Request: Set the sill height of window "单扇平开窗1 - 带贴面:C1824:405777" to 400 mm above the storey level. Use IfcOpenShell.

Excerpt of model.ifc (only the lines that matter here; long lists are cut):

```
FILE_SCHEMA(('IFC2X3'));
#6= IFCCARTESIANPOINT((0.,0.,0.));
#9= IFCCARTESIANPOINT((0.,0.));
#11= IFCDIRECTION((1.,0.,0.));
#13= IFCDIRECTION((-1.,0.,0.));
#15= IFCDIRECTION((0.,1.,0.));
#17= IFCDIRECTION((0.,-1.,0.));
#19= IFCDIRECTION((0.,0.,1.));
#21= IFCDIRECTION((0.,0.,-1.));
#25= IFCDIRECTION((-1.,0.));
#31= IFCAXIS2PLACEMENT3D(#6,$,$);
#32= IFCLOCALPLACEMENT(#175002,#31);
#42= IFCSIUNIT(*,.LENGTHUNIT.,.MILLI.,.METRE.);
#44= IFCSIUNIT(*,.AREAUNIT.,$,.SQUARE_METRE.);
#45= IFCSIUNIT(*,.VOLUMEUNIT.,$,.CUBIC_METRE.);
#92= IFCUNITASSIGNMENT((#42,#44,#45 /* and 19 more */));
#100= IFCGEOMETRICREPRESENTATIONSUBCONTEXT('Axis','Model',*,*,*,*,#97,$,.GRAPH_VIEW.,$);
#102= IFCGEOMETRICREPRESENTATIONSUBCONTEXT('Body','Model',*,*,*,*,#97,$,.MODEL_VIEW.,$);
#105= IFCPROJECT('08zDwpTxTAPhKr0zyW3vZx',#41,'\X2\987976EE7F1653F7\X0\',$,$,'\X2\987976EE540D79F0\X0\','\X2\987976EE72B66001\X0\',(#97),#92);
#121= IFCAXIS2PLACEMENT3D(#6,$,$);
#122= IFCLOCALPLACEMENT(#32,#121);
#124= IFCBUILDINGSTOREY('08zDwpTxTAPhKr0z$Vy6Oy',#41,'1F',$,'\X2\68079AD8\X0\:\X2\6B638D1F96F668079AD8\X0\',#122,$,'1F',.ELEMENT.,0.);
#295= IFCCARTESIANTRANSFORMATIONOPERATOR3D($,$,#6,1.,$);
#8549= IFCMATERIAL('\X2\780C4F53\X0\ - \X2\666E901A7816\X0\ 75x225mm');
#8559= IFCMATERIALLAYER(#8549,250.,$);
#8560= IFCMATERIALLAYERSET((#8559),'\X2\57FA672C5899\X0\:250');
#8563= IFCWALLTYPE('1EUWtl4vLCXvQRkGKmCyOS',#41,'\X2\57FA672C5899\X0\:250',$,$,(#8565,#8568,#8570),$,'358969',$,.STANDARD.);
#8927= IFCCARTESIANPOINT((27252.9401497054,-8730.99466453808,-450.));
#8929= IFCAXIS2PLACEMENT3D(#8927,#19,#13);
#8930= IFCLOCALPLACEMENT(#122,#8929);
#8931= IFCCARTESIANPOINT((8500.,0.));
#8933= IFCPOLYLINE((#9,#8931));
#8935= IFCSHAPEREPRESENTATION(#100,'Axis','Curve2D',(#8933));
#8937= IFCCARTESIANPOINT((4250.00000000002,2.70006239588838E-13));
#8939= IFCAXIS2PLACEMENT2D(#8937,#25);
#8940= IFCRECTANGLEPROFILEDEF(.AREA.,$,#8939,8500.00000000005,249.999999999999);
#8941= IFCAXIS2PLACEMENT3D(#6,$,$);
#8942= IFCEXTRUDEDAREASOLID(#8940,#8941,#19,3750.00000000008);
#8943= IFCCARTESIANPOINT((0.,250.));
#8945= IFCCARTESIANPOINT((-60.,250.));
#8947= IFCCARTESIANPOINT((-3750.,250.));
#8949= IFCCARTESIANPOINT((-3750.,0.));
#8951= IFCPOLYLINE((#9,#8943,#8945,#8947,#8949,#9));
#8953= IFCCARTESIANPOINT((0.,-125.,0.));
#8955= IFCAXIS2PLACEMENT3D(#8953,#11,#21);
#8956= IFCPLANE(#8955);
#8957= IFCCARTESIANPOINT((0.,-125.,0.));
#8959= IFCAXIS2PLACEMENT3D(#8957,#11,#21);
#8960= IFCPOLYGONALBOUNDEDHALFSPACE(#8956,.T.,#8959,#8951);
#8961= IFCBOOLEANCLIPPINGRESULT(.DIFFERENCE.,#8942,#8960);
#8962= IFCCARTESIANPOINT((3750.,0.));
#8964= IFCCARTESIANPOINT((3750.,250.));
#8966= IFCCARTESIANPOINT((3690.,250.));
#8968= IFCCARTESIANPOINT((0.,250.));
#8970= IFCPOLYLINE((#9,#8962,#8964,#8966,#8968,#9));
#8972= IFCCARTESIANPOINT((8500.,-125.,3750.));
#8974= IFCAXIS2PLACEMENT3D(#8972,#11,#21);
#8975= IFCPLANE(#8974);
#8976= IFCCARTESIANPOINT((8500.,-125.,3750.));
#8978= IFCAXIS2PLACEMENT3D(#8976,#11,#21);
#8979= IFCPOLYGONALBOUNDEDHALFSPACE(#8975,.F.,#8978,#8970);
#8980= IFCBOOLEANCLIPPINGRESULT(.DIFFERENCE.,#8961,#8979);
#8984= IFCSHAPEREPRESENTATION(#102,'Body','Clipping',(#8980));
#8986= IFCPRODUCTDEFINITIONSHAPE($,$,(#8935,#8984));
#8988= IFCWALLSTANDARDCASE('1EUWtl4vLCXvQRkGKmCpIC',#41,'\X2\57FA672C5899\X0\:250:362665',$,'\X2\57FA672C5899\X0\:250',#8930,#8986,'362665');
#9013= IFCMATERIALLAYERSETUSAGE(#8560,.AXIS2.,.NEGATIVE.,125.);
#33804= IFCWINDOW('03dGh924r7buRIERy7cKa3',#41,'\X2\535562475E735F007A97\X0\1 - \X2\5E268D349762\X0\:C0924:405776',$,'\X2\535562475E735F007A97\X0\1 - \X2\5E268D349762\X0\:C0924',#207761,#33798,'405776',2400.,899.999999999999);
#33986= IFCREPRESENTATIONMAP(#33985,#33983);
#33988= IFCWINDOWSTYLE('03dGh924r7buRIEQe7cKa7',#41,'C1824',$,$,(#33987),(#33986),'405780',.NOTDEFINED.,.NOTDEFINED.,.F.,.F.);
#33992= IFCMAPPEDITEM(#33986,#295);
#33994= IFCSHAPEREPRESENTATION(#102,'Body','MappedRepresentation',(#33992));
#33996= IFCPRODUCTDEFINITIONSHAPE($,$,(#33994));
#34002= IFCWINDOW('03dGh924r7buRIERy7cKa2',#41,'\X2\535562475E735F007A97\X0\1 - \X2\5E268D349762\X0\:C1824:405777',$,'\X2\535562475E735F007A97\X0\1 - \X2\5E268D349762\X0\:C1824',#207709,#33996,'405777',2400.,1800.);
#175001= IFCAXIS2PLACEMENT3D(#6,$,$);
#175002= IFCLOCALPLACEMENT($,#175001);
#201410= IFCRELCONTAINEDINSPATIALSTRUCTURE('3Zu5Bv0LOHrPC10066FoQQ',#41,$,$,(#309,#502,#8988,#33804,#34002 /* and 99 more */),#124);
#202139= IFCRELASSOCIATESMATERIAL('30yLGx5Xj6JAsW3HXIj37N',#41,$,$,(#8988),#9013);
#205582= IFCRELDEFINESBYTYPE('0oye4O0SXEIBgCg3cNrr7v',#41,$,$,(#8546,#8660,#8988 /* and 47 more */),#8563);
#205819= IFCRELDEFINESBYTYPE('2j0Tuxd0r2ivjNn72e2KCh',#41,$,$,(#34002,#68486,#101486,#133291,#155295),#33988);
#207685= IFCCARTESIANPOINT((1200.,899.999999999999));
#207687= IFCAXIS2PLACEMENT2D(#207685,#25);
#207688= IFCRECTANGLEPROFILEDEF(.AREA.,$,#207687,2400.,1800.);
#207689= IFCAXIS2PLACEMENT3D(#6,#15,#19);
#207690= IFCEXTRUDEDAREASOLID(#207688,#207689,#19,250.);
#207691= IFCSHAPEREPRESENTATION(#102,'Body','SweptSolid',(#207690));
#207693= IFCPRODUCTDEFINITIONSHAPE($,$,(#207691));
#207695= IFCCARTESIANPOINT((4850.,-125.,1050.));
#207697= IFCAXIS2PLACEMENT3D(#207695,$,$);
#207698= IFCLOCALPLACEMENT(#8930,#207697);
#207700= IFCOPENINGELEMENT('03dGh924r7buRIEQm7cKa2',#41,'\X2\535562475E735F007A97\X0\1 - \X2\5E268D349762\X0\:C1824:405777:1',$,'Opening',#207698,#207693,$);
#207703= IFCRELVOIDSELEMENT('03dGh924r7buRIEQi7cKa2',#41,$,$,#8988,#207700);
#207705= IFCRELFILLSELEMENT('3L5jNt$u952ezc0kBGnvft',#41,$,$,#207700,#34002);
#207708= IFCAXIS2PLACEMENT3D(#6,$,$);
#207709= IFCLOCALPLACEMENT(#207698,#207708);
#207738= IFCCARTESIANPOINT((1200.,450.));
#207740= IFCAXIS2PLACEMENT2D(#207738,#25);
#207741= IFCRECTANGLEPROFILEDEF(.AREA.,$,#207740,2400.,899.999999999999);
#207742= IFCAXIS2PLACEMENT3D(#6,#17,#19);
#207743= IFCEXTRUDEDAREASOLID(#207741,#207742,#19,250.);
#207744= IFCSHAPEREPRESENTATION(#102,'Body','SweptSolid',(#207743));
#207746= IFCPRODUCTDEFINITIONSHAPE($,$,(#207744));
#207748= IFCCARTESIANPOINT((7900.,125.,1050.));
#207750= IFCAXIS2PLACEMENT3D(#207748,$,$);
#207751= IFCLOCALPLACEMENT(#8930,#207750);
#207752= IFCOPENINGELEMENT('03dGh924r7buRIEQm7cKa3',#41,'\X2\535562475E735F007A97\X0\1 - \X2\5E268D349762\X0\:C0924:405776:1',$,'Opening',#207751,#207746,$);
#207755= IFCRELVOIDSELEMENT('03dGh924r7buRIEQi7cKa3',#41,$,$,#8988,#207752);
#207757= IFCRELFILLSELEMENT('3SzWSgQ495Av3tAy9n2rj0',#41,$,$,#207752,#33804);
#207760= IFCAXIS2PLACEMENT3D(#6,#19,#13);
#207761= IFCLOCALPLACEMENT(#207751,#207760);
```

```python
import numpy as np
import ifcopenshell
import ifcopenshell.api.geometry
import ifcopenshell.geom
import ifcopenshell.util.element
import ifcopenshell.util.placement
import ifcopenshell.util.shape
import ifcopenshell.util.unit

model = ifcopenshell.open("model.ifc")
unit_scale = ifcopenshell.util.unit.calculate_unit_scale(model)

window = model.by_id(34002)
opening = window.FillsVoids[0].RelatingOpeningElement
storey = ifcopenshell.util.element.get_container(window, ifc_class="IfcBuildingStorey")
level = ifcopenshell.util.placement.get_local_placement(storey.ObjectPlacement)[2, 3]

# The opening's origin need not be at the sill, so measure its lowest point.
shape = ifcopenshell.geom.create_shape(ifcopenshell.geom.settings(), opening)
bottom = ifcopenshell.util.shape.get_shape_bottom_elevation(shape, shape.geometry) / unit_scale
dz = level + 0.4 / unit_scale - bottom

shift = np.array([0.0, 0.0, dz])
# The window is placed relative to its opening, so it follows when the opening moves.
matrix = ifcopenshell.util.placement.get_local_placement(opening.ObjectPlacement)
matrix[:3, 3] += shift
ifcopenshell.api.geometry.edit_object_placement(
    model, product=opening, matrix=matrix, is_si=False, should_transform_children=True
)

print(f"moved by {dz * unit_scale:+.3f} m")

model.write("model_edited.ifc")
```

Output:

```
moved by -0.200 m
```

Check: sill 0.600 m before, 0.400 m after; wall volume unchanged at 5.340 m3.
